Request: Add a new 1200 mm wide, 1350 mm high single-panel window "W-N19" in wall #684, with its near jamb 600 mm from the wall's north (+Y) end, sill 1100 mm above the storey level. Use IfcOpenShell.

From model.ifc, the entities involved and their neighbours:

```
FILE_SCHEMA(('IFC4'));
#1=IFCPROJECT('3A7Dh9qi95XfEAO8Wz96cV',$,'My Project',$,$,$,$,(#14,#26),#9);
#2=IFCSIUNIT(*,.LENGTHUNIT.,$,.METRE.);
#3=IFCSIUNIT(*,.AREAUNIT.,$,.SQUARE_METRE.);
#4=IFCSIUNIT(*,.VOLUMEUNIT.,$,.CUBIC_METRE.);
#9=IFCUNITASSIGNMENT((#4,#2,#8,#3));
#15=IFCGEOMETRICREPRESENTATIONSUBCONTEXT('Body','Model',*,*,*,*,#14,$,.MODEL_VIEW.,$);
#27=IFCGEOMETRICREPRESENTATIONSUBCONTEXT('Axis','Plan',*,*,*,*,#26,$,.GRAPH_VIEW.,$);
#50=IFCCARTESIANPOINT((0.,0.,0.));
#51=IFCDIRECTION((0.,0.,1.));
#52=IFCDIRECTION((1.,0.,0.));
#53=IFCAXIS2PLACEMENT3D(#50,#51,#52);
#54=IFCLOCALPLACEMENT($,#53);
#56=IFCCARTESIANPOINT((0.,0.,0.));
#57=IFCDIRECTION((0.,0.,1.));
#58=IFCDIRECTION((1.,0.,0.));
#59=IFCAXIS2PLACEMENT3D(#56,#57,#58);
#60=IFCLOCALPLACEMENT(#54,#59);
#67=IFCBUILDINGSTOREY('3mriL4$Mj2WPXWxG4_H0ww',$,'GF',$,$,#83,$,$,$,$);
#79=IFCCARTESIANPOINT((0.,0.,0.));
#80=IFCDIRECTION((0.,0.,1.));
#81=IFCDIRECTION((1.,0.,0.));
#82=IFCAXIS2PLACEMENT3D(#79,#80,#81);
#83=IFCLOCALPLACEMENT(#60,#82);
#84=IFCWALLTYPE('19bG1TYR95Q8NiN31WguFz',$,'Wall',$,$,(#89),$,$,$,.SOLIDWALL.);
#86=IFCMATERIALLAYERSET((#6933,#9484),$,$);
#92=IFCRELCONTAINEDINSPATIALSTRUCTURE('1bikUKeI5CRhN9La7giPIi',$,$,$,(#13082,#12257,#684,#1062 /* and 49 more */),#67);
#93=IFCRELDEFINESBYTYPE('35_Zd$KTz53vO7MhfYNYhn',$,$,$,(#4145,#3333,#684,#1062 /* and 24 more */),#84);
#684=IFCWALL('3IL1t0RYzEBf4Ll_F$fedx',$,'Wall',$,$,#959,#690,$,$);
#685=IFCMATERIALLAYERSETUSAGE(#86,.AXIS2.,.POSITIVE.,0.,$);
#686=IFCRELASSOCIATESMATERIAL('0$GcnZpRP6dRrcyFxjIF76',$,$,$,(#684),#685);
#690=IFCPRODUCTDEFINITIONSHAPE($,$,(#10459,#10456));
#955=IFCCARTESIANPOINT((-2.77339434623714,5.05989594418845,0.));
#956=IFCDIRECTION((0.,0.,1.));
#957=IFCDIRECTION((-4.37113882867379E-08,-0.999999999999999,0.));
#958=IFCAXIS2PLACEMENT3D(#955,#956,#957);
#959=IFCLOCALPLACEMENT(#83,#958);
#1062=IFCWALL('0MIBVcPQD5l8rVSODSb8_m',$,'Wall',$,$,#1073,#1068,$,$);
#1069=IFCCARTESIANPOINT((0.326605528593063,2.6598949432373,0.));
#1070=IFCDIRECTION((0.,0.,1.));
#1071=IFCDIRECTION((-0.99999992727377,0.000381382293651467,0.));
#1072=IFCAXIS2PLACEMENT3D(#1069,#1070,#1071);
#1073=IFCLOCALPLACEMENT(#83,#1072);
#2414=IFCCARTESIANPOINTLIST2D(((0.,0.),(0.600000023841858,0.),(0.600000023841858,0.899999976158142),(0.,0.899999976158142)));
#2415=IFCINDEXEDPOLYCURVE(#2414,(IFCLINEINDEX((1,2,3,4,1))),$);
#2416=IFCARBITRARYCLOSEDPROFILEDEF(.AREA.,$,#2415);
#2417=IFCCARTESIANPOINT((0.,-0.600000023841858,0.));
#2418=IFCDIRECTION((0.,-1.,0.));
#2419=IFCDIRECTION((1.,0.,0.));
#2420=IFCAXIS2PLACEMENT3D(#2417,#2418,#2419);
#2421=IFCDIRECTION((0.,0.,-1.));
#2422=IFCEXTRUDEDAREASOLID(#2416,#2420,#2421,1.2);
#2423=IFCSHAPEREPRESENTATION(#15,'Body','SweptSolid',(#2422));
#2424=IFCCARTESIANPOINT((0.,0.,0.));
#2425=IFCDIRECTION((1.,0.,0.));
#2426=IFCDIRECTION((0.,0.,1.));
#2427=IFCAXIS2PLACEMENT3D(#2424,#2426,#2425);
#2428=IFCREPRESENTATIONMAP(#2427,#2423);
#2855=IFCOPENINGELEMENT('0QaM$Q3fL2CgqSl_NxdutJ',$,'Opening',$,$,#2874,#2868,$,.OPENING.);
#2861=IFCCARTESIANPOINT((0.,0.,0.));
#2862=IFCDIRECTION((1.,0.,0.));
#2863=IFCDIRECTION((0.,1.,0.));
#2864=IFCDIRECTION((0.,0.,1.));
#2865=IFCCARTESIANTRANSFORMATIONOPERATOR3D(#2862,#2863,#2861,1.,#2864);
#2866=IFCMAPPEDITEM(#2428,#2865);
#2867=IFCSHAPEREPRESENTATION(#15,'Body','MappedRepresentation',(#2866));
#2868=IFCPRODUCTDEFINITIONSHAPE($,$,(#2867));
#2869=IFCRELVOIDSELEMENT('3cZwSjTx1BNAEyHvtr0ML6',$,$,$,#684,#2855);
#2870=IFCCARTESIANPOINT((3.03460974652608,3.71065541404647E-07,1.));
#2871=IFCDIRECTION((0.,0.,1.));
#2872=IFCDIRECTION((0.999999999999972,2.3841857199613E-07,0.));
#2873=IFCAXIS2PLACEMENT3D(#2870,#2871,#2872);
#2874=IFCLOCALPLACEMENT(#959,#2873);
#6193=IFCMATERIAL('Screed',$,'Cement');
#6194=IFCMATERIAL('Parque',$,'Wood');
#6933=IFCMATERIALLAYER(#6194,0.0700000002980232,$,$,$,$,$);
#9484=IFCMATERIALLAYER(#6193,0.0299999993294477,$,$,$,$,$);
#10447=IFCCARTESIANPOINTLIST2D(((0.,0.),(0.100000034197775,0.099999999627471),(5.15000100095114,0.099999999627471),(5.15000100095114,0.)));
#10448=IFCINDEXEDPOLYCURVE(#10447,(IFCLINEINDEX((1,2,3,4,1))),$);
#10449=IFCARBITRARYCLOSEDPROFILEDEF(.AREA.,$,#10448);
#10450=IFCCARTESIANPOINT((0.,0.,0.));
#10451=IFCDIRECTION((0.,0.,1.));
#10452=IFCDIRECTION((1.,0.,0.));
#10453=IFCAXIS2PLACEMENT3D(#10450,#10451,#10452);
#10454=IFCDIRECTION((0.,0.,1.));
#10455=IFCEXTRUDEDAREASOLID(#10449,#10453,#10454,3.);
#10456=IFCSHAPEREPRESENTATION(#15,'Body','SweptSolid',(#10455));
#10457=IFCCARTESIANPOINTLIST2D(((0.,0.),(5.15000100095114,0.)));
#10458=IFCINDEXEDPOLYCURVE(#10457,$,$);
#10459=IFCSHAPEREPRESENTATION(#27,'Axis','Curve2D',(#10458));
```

```python
import numpy as np
import ifcopenshell
import ifcopenshell.api.feature
import ifcopenshell.api.geometry
import ifcopenshell.api.root
import ifcopenshell.api.spatial
import ifcopenshell.geom
import ifcopenshell.util.element
import ifcopenshell.util.placement
import ifcopenshell.util.representation
import ifcopenshell.util.shape
import ifcopenshell.util.unit

model = ifcopenshell.open("model.ifc")
unit_scale = ifcopenshell.util.unit.calculate_unit_scale(model)
settings = ifcopenshell.geom.settings()


def volume(element):
    """Net volume in cubic metres, openings subtracted."""
    shape = ifcopenshell.geom.create_shape(settings, element)
    return ifcopenshell.util.shape.get_volume(shape.geometry)


wall = model.by_guid("3IL1t0RYzEBf4Ll_F$fedx")
storey = ifcopenshell.util.element.get_container(wall, ifc_class="IfcBuildingStorey")
context = ifcopenshell.util.representation.get_context(model, "Model", "Body", "MODEL_VIEW")
before = volume(wall)

width, height, from_end, sill = 1.2, 1.35, 0.6, 1.1  # metres

# The wall runs along its own X axis, and the end named is its -X end.
wall_shape = ifcopenshell.geom.create_shape(settings, wall)
x, y, z = ifcopenshell.util.shape.get_vertices(wall_shape.geometry).T
start = x.min() + from_end
face, thickness = float(y.min()), float(y.max() - y.min())
wall_matrix = ifcopenshell.util.placement.get_local_placement(wall.ObjectPlacement)
level = ifcopenshell.util.placement.get_local_placement(storey.ObjectPlacement)[2, 3]


def in_wall(x, y):
    """Placement at x, y metres in the wall's axes, at sill height."""
    matrix = wall_matrix.copy()
    matrix[:, 3] = wall_matrix @ np.array([x / unit_scale, y / unit_scale, 0.0, 1.0])
    matrix[2, 3] = level + sill / unit_scale
    return matrix


# Opening: a box that overshoots both wall faces by 50 mm.
opening = ifcopenshell.api.root.create_entity(model, ifc_class="IfcOpeningElement", predefined_type="OPENING")
box = ifcopenshell.api.geometry.add_wall_representation(
    model, context=context, length=width, height=height, thickness=thickness + 0.1
)
ifcopenshell.api.geometry.assign_representation(model, product=opening, representation=box)
ifcopenshell.api.geometry.edit_object_placement(model, product=opening, matrix=in_wall(start, face - 0.05), is_si=False)
ifcopenshell.api.feature.add_feature(model, feature=opening, element=wall)

window = ifcopenshell.api.root.create_entity(model, ifc_class="IfcWindow", name="W-N19", predefined_type="WINDOW")
window.OverallWidth, window.OverallHeight = width / unit_scale, height / unit_scale
window.PartitioningType = "SINGLE_PANEL"
body = ifcopenshell.api.geometry.add_window_representation(
    model,
    context=context,
    overall_width=window.OverallWidth,
    overall_height=window.OverallHeight,
    partition_type="SINGLE_PANEL",
)
ifcopenshell.api.geometry.assign_representation(model, product=window, representation=body)
ifcopenshell.api.spatial.assign_container(model, products=[window], relating_structure=storey)
ifcopenshell.api.feature.add_filling(model, opening=opening, element=window)

# Centre the window in the wall's thickness.
ifcopenshell.api.geometry.edit_object_placement(model, product=window, matrix=in_wall(start, face), is_si=False)
window_shape = ifcopenshell.geom.create_shape(settings, window)
depth = ifcopenshell.util.shape.get_vertices(window_shape.geometry)[:, 1]
offset = face + thickness / 2 - (depth.min() + depth.max()) / 2
ifcopenshell.api.geometry.edit_object_placement(model, product=window, matrix=in_wall(start, offset), is_si=False)

after = volume(wall)

print(f"wall volume {before:.3f} -> {after:.3f} m3")

model.write("model_edited.ifc")
```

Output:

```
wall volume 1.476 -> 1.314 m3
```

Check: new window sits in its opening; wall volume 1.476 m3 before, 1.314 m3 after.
